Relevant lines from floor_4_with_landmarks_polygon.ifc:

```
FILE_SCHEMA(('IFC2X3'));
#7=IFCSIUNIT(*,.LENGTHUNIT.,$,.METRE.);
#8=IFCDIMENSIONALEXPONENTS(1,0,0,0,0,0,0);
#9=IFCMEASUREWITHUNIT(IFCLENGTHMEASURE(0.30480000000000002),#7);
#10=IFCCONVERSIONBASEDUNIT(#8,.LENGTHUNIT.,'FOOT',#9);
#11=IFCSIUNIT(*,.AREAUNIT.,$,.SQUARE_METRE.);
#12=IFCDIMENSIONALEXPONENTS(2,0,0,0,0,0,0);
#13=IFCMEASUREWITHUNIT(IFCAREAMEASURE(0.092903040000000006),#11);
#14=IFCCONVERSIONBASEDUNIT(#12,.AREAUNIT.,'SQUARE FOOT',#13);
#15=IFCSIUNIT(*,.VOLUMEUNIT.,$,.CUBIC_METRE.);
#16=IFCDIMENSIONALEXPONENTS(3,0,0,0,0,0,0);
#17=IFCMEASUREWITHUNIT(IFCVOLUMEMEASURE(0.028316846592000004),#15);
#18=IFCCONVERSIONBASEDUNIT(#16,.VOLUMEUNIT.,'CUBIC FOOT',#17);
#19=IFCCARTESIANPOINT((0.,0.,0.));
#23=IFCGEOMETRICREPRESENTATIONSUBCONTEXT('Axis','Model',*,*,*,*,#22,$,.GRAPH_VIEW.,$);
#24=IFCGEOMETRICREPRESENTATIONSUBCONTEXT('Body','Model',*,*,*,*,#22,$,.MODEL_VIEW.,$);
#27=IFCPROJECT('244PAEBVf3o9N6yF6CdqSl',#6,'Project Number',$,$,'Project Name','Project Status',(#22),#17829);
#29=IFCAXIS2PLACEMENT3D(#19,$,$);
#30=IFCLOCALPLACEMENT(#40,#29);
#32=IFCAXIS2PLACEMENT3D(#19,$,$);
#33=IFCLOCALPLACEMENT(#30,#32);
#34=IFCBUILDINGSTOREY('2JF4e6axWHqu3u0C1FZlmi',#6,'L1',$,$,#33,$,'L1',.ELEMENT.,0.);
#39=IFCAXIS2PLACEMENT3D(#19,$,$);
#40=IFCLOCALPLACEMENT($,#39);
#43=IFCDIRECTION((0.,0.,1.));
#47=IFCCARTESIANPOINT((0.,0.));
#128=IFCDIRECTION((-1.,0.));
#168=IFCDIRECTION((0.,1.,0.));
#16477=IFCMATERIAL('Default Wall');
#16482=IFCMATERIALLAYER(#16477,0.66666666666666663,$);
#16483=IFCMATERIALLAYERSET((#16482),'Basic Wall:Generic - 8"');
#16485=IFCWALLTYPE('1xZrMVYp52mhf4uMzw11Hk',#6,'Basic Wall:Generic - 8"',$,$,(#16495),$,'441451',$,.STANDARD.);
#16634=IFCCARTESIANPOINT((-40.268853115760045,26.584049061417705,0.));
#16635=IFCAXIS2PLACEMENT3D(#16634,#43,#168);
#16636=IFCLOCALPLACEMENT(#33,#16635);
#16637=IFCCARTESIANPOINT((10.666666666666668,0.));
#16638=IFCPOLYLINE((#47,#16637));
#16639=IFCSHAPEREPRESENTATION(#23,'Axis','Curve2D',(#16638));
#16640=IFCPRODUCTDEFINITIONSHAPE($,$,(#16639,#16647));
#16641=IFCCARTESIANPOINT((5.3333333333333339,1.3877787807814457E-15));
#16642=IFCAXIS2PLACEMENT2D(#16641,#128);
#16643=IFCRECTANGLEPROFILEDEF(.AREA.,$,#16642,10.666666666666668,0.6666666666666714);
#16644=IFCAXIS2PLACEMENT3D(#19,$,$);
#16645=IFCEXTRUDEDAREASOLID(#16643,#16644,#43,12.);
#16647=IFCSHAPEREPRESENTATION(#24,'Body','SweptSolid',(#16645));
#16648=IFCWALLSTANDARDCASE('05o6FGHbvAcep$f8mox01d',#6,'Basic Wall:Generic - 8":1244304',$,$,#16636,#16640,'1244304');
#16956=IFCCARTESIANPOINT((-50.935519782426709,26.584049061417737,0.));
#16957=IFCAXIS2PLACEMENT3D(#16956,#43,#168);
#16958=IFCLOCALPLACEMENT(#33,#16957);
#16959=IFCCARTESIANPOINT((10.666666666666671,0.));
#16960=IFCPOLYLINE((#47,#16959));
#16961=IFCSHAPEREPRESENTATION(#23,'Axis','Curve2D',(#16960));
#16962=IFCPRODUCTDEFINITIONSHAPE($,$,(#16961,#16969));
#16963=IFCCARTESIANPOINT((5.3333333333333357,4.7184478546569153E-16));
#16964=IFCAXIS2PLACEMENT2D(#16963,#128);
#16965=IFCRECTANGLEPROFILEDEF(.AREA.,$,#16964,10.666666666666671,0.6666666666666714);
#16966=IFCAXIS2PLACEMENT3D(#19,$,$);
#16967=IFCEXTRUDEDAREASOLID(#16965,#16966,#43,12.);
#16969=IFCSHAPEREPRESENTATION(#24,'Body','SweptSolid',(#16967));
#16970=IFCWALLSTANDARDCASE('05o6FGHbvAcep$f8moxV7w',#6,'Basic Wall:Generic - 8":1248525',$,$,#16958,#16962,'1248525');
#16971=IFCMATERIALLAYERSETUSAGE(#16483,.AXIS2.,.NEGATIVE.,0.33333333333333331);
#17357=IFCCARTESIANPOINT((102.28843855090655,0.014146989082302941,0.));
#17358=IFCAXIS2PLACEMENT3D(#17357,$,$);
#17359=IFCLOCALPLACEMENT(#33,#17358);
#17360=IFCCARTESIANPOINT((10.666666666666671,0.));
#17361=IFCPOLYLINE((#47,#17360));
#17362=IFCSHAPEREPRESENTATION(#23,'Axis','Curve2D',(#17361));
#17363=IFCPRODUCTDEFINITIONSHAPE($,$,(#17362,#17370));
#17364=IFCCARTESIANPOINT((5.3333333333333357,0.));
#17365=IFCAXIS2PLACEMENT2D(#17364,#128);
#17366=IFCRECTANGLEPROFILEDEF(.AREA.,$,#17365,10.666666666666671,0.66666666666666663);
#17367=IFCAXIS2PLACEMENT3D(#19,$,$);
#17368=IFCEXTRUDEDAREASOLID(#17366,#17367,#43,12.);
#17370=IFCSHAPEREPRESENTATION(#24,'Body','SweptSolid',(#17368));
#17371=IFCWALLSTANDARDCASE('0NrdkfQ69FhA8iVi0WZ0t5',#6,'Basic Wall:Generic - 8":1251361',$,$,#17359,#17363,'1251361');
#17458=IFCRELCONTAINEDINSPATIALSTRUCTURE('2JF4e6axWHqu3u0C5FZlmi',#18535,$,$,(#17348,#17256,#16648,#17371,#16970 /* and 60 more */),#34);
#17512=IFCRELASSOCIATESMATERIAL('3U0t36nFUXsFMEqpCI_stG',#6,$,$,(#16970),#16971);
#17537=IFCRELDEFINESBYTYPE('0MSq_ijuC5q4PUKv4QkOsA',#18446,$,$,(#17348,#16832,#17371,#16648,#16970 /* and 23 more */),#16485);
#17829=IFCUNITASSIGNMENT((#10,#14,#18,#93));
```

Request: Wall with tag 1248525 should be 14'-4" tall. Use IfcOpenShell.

```python
import ifcopenshell
import ifcopenshell.geom
import ifcopenshell.util.representation
import ifcopenshell.util.shape
import ifcopenshell.util.unit

model = ifcopenshell.open("floor_4_with_landmarks_polygon.ifc")
unit_scale = ifcopenshell.util.unit.calculate_unit_scale(model)
settings = ifcopenshell.geom.settings()


def volume(element):
    """Net volume in cubic metres, openings subtracted."""
    shape = ifcopenshell.geom.create_shape(settings, element)
    return ifcopenshell.util.shape.get_volume(shape.geometry)


wall = model.by_id(16970)
before = volume(wall)

body = ifcopenshell.util.representation.get_representation(wall, "Model", "Body")
solid = body.Items[0]
old_height = solid.Depth
solid.Depth = 172 * 0.0254 / unit_scale
after = volume(wall)

print(f"height {old_height:g} -> {solid.Depth:g}, volume {before:.3f} -> {after:.3f} m3")

model.write("floor_4_with_landmarks_polygon_updated.ifc")
```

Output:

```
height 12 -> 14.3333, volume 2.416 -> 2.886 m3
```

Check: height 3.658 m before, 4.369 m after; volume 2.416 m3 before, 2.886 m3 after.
